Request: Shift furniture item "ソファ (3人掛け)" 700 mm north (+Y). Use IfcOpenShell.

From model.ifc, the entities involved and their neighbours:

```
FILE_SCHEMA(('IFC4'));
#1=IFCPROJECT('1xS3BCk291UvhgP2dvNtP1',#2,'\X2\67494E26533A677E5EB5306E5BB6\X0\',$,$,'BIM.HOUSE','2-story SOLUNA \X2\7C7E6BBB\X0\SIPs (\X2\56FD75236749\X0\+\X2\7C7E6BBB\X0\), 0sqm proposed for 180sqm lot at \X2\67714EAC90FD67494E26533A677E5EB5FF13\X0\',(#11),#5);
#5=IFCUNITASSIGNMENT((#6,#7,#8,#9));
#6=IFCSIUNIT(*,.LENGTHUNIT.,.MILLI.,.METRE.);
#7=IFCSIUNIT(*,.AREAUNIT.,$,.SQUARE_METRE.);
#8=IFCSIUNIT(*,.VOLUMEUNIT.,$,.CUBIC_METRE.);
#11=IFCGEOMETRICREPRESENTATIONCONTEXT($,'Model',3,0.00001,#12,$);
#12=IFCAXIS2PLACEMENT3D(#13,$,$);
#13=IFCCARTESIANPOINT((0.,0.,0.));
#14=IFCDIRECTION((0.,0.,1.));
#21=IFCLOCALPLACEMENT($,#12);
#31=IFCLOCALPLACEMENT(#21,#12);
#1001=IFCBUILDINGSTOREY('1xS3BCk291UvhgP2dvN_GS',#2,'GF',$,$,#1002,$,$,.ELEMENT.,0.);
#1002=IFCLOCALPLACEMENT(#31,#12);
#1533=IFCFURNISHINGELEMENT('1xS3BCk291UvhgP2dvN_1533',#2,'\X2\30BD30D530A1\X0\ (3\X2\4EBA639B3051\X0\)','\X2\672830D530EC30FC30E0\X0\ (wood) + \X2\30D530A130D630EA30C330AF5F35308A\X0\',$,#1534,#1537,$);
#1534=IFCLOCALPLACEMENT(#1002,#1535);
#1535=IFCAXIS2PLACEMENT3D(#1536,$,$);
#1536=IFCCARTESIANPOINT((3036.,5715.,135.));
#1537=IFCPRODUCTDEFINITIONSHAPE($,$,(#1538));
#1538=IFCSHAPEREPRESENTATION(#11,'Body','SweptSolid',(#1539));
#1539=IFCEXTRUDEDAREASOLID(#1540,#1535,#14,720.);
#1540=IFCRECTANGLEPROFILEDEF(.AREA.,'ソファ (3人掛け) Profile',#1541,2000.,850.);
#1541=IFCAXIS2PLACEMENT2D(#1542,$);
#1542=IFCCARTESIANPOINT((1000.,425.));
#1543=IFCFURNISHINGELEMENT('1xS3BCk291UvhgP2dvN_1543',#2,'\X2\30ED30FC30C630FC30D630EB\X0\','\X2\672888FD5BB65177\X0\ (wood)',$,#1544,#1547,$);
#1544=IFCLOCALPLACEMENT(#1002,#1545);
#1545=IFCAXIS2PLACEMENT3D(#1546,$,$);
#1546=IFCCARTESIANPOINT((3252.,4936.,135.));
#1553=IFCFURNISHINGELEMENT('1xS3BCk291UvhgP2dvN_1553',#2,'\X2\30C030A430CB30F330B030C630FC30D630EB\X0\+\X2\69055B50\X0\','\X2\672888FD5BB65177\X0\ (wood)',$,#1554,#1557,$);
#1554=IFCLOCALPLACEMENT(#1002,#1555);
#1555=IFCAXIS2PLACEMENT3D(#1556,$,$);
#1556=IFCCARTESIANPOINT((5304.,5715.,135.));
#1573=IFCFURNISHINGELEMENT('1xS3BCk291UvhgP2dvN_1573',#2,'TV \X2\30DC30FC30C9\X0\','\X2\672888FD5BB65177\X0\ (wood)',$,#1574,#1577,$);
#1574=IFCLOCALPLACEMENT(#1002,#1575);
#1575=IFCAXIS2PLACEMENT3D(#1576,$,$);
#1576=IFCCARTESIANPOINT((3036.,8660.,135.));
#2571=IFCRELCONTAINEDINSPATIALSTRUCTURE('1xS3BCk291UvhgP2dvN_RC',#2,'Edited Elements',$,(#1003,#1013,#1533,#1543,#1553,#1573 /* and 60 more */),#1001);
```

```python
import ifcopenshell
import ifcopenshell.api.geometry
import ifcopenshell.util.placement

model = ifcopenshell.open("model.ifc")

item = model.by_id(1533)
matrix = ifcopenshell.util.placement.get_local_placement(item.ObjectPlacement)
matrix[1, 3] += 700.0
ifcopenshell.api.geometry.edit_object_placement(model, product=item, matrix=matrix, is_si=False)

print(ifcopenshell.util.placement.get_local_placement(item.ObjectPlacement).round(3) + 0.0)

model.write("model_rev.ifc")
```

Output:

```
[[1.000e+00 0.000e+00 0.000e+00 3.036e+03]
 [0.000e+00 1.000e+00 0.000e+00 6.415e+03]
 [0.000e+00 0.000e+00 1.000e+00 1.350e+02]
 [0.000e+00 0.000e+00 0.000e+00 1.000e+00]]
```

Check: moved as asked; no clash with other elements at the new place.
